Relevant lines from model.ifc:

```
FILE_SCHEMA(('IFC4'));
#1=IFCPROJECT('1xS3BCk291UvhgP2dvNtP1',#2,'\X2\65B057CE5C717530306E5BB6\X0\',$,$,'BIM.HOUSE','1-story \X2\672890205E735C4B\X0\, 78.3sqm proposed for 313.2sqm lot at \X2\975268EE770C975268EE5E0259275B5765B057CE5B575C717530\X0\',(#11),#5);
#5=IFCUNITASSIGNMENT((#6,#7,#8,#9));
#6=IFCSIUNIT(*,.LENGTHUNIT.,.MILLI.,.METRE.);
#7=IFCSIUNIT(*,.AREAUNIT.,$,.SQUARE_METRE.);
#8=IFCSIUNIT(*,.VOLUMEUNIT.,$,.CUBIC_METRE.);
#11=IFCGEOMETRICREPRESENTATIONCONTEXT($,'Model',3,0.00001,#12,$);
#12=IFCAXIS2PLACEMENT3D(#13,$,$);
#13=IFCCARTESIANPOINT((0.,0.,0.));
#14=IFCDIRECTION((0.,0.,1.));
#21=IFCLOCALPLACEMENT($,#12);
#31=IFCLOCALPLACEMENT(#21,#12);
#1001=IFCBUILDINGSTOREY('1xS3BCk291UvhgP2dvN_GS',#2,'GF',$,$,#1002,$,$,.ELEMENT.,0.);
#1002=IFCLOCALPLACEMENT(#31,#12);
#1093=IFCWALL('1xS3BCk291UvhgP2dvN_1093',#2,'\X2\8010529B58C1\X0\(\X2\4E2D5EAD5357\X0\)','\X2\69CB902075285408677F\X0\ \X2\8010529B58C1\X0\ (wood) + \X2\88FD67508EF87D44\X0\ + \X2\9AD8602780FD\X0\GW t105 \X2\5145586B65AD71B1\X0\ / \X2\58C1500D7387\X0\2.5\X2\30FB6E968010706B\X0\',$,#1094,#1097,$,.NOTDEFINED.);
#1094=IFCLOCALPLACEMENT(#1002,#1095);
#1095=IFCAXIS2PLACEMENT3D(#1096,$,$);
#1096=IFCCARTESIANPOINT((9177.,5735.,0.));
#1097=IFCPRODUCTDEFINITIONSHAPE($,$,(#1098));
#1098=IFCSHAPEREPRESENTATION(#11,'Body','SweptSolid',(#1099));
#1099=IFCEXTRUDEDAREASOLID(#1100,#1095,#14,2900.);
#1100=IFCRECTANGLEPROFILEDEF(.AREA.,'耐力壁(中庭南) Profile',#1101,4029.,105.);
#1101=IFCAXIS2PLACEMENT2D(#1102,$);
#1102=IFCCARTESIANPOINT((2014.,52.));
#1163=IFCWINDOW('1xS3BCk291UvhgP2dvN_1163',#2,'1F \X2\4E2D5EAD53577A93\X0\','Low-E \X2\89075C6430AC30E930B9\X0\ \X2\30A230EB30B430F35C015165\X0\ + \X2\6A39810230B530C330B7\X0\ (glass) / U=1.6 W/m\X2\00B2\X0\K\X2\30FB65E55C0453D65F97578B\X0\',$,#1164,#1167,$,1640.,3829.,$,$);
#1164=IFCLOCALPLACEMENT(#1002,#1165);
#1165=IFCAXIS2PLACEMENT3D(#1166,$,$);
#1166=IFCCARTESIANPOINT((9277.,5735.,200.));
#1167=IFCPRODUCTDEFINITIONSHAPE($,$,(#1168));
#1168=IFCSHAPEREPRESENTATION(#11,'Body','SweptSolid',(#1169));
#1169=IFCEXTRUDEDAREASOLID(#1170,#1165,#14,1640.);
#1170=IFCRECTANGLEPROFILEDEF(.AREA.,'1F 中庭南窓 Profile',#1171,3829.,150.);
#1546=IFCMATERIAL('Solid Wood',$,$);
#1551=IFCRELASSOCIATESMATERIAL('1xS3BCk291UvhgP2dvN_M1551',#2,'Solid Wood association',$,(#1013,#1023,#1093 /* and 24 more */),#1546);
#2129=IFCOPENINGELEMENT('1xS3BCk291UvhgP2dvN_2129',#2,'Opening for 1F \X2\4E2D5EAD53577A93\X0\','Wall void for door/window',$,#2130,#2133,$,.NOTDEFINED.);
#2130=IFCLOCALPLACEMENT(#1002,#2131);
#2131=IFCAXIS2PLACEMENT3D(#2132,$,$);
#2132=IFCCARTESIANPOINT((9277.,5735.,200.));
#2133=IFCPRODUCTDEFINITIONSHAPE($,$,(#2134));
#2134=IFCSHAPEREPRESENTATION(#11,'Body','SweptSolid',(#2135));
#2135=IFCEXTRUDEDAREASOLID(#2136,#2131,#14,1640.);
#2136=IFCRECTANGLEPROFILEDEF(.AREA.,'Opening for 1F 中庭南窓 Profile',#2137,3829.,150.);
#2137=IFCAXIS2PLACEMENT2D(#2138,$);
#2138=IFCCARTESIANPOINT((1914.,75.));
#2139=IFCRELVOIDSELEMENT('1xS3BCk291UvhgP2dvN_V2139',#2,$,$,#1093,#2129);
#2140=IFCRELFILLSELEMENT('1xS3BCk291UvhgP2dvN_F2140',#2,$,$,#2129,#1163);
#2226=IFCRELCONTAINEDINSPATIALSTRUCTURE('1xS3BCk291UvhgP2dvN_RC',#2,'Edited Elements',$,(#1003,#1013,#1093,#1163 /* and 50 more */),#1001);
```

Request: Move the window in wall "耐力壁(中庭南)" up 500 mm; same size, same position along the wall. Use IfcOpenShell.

```python
import numpy as np
import ifcopenshell
import ifcopenshell.api.geometry
import ifcopenshell.util.placement
import ifcopenshell.util.unit

model = ifcopenshell.open("model.ifc")
unit_scale = ifcopenshell.util.unit.calculate_unit_scale(model)

window = model.by_id(1163)
opening = window.FillsVoids[0].RelatingOpeningElement
dz = 0.5 / unit_scale

shift = np.array([0.0, 0.0, dz])
# The window is not placed relative to its opening, so move both.
for product in (opening, window):
    matrix = ifcopenshell.util.placement.get_local_placement(product.ObjectPlacement)
    matrix[:3, 3] += shift
    ifcopenshell.api.geometry.edit_object_placement(model, product=product, matrix=matrix, is_si=False)

print(f"moved by {dz * unit_scale:+.3f} m")

model.write("model_updated.ifc")
```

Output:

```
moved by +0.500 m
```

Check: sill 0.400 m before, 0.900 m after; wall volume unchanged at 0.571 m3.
